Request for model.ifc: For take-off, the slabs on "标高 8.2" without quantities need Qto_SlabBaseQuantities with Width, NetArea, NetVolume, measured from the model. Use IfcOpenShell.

First a look at what the model holds.

```python
import ifcopenshell
import ifcopenshell.util.element
import ifcopenshell.util.unit

model = ifcopenshell.open("model.ifc")
print(model.schema)
for unit_type in ("LENGTHUNIT", "AREAUNIT", "VOLUMEUNIT"):
    print(unit_type, ifcopenshell.util.unit.calculate_unit_scale(model, unit_type))
storey = next(s for s in model.by_type("IfcBuildingStorey") if s.Name == "标高 8.2")
slabs = [e for e in ifcopenshell.util.element.get_decomposition(storey) if e.is_a("IfcSlab")]
for e in sorted(slabs, key=lambda e: e.id()):
    print(e.id(), e.is_a(), e.Name, list(ifcopenshell.util.element.get_psets(e, qtos_only=True)), sep=" | ")
```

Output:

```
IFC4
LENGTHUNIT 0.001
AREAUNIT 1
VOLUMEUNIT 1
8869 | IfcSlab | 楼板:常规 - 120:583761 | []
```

```python
import ifcopenshell
import ifcopenshell.api.pset
import ifcopenshell.geom
import ifcopenshell.util.element
import ifcopenshell.util.shape
import ifcopenshell.util.unit

model = ifcopenshell.open("model.ifc")
unit_scale = ifcopenshell.util.unit.calculate_unit_scale(model)
area_scale = ifcopenshell.util.unit.calculate_unit_scale(model, "AREAUNIT")
volume_scale = ifcopenshell.util.unit.calculate_unit_scale(model, "VOLUMEUNIT")
settings = ifcopenshell.geom.settings()

storey = next(s for s in model.by_type("IfcBuildingStorey") if s.Name == "标高 8.2")
slabs = [e for e in ifcopenshell.util.element.get_decomposition(storey) if e.is_a("IfcSlab")]

for e in sorted(slabs, key=lambda e: e.id()):
    if ifcopenshell.util.element.get_psets(e, qtos_only=True, should_inherit=False):
        continue
    # Geometry comes back in metres, in the element's own axes.
    shape = ifcopenshell.geom.create_shape(settings, e)
    values = {
        "Width": ifcopenshell.util.shape.get_z(shape.geometry) / unit_scale,
        "NetArea": ifcopenshell.util.shape.get_footprint_area(shape.geometry) / area_scale,
        "NetVolume": ifcopenshell.util.shape.get_volume(shape.geometry) / volume_scale,
    }
    qto = ifcopenshell.api.pset.add_qto(model, product=e, name="Qto_SlabBaseQuantities")
    ifcopenshell.api.pset.edit_qto(model, qto=qto, properties=values)
    print(e.id(), {k: round(v, 3) for k, v in values.items()})

model.write("model_updated.ifc")
```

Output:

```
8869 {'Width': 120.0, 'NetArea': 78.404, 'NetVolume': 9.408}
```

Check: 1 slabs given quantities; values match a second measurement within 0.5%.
